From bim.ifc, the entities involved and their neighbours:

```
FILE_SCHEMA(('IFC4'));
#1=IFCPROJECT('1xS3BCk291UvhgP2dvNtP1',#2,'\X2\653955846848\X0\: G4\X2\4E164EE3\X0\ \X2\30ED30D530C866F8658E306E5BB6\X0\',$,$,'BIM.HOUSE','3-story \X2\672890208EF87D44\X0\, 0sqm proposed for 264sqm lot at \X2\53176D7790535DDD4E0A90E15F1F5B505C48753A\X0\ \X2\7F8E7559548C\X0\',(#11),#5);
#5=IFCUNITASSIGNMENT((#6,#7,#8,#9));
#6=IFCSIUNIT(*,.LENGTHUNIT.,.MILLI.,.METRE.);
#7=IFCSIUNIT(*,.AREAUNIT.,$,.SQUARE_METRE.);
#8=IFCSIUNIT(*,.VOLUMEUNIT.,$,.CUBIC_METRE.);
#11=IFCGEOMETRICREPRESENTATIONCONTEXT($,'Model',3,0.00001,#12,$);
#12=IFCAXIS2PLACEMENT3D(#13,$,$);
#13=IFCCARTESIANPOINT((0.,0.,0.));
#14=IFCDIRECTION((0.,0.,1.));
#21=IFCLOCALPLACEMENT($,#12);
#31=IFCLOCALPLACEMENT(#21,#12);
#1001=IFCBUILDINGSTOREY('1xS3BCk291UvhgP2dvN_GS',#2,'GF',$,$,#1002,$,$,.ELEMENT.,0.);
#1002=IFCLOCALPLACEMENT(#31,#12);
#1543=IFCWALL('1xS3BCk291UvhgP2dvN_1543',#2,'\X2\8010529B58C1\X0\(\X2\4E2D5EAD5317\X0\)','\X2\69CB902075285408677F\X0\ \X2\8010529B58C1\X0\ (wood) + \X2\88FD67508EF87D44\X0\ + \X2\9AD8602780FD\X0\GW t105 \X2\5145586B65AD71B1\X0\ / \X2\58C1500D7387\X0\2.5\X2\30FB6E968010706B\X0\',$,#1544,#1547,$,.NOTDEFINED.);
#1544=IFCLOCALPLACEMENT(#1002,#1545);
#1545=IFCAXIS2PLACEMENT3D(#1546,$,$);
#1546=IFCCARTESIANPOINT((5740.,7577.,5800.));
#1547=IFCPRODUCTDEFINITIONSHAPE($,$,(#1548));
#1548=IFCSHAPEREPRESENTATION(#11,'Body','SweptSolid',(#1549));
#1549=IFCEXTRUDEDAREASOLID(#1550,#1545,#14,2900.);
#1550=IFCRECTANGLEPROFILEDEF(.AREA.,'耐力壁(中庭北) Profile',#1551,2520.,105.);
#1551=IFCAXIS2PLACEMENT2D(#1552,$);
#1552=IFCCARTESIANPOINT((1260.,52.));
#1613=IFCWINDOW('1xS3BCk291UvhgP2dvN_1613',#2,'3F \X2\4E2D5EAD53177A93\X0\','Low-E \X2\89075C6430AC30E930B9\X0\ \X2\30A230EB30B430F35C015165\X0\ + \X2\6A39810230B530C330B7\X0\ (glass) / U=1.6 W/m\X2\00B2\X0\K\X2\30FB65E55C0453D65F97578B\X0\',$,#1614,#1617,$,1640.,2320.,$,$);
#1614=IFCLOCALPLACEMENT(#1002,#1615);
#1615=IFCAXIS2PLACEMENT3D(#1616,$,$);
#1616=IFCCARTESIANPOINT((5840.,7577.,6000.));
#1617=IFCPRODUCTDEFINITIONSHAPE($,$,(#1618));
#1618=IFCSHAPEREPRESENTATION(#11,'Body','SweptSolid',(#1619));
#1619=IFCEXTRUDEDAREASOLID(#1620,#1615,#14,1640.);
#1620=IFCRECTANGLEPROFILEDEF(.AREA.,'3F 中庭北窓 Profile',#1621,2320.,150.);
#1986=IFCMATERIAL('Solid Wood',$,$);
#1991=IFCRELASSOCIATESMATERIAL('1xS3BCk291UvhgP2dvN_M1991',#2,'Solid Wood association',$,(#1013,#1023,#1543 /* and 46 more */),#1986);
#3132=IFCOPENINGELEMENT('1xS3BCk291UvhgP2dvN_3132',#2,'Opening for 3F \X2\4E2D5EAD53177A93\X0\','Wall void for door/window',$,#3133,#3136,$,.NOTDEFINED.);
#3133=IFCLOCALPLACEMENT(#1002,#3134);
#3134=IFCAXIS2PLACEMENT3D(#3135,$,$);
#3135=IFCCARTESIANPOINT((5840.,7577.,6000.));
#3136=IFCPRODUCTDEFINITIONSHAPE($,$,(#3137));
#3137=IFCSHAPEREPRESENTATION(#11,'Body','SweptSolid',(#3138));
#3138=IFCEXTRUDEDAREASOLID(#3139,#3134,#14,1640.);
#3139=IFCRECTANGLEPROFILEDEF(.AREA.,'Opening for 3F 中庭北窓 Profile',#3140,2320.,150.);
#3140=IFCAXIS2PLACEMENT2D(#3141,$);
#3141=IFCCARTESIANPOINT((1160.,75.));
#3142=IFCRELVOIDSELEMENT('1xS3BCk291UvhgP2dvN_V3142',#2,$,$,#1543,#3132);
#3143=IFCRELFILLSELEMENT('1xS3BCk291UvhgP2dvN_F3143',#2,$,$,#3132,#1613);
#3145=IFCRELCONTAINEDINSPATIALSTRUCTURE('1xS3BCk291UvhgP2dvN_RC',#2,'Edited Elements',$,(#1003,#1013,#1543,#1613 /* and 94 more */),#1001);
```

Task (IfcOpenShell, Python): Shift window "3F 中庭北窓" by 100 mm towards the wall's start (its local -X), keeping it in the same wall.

```python
import ifcopenshell
import ifcopenshell.api.geometry
import ifcopenshell.util.placement
import ifcopenshell.util.unit

model = ifcopenshell.open("bim.ifc")
unit_scale = ifcopenshell.util.unit.calculate_unit_scale(model)

window = model.by_id(1613)
opening = window.FillsVoids[0].RelatingOpeningElement
wall = opening.VoidsElements[0].RelatingBuildingElement

wall_matrix = ifcopenshell.util.placement.get_local_placement(wall.ObjectPlacement)
shift = wall_matrix[:3, 0] * -0.1 / unit_scale
before = ifcopenshell.util.placement.get_local_placement(window.ObjectPlacement)[:3, 3].copy()

# The window is not placed relative to its opening, so move both.
for product in (opening, window):
    matrix = ifcopenshell.util.placement.get_local_placement(product.ObjectPlacement)
    matrix[:3, 3] += shift
    ifcopenshell.api.geometry.edit_object_placement(model, product=product, matrix=matrix, is_si=False)

after = ifcopenshell.util.placement.get_local_placement(window.ObjectPlacement)[:3, 3]
print("window moved by", (after - before).round(3) + 0.0)

model.write("bim_rev.ifc")
```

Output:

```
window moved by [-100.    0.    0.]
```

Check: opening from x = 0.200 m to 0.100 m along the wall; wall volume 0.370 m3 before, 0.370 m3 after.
